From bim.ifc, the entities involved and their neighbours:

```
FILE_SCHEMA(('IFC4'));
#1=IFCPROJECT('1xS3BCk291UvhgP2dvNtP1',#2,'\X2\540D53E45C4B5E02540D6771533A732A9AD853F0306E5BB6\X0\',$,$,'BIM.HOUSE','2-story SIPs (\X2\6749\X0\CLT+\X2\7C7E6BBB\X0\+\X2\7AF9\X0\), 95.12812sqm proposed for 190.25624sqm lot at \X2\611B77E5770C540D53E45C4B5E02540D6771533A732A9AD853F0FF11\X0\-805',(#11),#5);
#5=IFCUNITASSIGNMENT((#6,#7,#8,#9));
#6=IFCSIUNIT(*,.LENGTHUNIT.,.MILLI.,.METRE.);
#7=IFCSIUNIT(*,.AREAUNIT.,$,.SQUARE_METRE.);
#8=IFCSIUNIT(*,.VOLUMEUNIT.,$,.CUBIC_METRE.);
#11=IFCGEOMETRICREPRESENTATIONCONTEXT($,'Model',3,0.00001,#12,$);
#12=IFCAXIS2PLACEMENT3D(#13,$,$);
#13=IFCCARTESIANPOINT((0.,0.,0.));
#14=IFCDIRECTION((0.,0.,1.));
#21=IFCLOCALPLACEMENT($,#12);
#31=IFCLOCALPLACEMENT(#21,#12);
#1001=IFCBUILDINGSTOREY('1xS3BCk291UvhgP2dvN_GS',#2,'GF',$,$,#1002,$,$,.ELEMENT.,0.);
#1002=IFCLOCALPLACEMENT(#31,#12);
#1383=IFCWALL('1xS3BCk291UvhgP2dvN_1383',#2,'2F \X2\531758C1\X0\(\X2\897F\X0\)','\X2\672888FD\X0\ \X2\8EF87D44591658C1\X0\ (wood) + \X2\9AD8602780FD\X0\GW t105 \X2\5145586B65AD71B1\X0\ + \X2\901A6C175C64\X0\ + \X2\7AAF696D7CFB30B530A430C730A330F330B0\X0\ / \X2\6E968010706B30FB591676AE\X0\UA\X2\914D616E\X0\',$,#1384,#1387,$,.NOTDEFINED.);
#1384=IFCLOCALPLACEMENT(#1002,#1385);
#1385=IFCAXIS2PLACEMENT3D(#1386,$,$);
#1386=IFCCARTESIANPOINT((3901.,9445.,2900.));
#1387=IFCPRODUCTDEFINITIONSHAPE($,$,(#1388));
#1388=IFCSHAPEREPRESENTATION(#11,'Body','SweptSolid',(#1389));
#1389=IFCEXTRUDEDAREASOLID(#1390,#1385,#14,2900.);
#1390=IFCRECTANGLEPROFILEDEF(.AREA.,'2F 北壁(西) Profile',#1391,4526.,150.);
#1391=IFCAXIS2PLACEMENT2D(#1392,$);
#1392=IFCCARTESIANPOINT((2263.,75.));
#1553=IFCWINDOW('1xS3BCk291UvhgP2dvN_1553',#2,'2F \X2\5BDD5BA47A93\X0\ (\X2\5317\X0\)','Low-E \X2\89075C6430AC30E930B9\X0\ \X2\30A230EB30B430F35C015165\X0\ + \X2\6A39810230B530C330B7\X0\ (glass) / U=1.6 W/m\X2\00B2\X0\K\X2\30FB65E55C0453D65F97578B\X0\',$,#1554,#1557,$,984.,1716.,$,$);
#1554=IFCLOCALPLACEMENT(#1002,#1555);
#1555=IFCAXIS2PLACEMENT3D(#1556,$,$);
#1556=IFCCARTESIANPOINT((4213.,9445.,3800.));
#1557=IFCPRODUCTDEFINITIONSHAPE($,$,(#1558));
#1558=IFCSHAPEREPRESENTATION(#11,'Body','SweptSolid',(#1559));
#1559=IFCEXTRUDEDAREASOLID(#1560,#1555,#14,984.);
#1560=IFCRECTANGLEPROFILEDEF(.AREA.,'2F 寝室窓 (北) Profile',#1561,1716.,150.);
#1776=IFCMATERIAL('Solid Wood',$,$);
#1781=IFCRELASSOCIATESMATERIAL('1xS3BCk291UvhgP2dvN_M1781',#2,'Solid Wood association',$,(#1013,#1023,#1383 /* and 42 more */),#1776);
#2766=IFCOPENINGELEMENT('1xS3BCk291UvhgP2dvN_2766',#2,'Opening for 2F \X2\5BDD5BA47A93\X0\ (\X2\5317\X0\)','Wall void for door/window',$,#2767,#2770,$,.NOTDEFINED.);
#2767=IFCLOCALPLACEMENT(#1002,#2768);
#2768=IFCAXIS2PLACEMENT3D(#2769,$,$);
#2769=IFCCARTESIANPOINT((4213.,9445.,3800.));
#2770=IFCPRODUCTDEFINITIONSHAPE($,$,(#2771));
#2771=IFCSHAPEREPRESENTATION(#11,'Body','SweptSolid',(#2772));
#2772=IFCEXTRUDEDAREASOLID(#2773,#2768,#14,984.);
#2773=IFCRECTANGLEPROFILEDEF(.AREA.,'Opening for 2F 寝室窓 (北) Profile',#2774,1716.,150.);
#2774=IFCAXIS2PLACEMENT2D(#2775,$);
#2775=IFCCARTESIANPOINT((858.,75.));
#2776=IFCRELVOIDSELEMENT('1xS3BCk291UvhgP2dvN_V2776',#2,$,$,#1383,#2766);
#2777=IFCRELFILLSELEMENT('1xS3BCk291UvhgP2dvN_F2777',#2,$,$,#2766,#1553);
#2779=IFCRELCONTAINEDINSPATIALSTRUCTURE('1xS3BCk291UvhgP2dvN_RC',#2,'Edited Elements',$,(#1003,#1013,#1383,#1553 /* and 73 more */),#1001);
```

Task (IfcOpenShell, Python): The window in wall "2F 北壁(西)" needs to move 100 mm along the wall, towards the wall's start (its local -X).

```python
import ifcopenshell
import ifcopenshell.api.geometry
import ifcopenshell.util.placement

model = ifcopenshell.open("bim.ifc")

window = model.by_guid("1xS3BCk291UvhgP2dvN_1553")
opening = window.FillsVoids[0].RelatingOpeningElement
wall = opening.VoidsElements[0].RelatingBuildingElement

wall_matrix = ifcopenshell.util.placement.get_local_placement(wall.ObjectPlacement)
shift = wall_matrix[:3, 0] * -100.0
before = ifcopenshell.util.placement.get_local_placement(window.ObjectPlacement)[:3, 3].copy()

# The window is not placed relative to its opening, so move both.
for product in (opening, window):
    matrix = ifcopenshell.util.placement.get_local_placement(product.ObjectPlacement)
    matrix[:3, 3] += shift
    ifcopenshell.api.geometry.edit_object_placement(model, product=product, matrix=matrix, is_si=False)

after = ifcopenshell.util.placement.get_local_placement(window.ObjectPlacement)[:3, 3]
print("window moved by", (after - before).round(3) + 0.0)

model.write("bim_rev.ifc")
```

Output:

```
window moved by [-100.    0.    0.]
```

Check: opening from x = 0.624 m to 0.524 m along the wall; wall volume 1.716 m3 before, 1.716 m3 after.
